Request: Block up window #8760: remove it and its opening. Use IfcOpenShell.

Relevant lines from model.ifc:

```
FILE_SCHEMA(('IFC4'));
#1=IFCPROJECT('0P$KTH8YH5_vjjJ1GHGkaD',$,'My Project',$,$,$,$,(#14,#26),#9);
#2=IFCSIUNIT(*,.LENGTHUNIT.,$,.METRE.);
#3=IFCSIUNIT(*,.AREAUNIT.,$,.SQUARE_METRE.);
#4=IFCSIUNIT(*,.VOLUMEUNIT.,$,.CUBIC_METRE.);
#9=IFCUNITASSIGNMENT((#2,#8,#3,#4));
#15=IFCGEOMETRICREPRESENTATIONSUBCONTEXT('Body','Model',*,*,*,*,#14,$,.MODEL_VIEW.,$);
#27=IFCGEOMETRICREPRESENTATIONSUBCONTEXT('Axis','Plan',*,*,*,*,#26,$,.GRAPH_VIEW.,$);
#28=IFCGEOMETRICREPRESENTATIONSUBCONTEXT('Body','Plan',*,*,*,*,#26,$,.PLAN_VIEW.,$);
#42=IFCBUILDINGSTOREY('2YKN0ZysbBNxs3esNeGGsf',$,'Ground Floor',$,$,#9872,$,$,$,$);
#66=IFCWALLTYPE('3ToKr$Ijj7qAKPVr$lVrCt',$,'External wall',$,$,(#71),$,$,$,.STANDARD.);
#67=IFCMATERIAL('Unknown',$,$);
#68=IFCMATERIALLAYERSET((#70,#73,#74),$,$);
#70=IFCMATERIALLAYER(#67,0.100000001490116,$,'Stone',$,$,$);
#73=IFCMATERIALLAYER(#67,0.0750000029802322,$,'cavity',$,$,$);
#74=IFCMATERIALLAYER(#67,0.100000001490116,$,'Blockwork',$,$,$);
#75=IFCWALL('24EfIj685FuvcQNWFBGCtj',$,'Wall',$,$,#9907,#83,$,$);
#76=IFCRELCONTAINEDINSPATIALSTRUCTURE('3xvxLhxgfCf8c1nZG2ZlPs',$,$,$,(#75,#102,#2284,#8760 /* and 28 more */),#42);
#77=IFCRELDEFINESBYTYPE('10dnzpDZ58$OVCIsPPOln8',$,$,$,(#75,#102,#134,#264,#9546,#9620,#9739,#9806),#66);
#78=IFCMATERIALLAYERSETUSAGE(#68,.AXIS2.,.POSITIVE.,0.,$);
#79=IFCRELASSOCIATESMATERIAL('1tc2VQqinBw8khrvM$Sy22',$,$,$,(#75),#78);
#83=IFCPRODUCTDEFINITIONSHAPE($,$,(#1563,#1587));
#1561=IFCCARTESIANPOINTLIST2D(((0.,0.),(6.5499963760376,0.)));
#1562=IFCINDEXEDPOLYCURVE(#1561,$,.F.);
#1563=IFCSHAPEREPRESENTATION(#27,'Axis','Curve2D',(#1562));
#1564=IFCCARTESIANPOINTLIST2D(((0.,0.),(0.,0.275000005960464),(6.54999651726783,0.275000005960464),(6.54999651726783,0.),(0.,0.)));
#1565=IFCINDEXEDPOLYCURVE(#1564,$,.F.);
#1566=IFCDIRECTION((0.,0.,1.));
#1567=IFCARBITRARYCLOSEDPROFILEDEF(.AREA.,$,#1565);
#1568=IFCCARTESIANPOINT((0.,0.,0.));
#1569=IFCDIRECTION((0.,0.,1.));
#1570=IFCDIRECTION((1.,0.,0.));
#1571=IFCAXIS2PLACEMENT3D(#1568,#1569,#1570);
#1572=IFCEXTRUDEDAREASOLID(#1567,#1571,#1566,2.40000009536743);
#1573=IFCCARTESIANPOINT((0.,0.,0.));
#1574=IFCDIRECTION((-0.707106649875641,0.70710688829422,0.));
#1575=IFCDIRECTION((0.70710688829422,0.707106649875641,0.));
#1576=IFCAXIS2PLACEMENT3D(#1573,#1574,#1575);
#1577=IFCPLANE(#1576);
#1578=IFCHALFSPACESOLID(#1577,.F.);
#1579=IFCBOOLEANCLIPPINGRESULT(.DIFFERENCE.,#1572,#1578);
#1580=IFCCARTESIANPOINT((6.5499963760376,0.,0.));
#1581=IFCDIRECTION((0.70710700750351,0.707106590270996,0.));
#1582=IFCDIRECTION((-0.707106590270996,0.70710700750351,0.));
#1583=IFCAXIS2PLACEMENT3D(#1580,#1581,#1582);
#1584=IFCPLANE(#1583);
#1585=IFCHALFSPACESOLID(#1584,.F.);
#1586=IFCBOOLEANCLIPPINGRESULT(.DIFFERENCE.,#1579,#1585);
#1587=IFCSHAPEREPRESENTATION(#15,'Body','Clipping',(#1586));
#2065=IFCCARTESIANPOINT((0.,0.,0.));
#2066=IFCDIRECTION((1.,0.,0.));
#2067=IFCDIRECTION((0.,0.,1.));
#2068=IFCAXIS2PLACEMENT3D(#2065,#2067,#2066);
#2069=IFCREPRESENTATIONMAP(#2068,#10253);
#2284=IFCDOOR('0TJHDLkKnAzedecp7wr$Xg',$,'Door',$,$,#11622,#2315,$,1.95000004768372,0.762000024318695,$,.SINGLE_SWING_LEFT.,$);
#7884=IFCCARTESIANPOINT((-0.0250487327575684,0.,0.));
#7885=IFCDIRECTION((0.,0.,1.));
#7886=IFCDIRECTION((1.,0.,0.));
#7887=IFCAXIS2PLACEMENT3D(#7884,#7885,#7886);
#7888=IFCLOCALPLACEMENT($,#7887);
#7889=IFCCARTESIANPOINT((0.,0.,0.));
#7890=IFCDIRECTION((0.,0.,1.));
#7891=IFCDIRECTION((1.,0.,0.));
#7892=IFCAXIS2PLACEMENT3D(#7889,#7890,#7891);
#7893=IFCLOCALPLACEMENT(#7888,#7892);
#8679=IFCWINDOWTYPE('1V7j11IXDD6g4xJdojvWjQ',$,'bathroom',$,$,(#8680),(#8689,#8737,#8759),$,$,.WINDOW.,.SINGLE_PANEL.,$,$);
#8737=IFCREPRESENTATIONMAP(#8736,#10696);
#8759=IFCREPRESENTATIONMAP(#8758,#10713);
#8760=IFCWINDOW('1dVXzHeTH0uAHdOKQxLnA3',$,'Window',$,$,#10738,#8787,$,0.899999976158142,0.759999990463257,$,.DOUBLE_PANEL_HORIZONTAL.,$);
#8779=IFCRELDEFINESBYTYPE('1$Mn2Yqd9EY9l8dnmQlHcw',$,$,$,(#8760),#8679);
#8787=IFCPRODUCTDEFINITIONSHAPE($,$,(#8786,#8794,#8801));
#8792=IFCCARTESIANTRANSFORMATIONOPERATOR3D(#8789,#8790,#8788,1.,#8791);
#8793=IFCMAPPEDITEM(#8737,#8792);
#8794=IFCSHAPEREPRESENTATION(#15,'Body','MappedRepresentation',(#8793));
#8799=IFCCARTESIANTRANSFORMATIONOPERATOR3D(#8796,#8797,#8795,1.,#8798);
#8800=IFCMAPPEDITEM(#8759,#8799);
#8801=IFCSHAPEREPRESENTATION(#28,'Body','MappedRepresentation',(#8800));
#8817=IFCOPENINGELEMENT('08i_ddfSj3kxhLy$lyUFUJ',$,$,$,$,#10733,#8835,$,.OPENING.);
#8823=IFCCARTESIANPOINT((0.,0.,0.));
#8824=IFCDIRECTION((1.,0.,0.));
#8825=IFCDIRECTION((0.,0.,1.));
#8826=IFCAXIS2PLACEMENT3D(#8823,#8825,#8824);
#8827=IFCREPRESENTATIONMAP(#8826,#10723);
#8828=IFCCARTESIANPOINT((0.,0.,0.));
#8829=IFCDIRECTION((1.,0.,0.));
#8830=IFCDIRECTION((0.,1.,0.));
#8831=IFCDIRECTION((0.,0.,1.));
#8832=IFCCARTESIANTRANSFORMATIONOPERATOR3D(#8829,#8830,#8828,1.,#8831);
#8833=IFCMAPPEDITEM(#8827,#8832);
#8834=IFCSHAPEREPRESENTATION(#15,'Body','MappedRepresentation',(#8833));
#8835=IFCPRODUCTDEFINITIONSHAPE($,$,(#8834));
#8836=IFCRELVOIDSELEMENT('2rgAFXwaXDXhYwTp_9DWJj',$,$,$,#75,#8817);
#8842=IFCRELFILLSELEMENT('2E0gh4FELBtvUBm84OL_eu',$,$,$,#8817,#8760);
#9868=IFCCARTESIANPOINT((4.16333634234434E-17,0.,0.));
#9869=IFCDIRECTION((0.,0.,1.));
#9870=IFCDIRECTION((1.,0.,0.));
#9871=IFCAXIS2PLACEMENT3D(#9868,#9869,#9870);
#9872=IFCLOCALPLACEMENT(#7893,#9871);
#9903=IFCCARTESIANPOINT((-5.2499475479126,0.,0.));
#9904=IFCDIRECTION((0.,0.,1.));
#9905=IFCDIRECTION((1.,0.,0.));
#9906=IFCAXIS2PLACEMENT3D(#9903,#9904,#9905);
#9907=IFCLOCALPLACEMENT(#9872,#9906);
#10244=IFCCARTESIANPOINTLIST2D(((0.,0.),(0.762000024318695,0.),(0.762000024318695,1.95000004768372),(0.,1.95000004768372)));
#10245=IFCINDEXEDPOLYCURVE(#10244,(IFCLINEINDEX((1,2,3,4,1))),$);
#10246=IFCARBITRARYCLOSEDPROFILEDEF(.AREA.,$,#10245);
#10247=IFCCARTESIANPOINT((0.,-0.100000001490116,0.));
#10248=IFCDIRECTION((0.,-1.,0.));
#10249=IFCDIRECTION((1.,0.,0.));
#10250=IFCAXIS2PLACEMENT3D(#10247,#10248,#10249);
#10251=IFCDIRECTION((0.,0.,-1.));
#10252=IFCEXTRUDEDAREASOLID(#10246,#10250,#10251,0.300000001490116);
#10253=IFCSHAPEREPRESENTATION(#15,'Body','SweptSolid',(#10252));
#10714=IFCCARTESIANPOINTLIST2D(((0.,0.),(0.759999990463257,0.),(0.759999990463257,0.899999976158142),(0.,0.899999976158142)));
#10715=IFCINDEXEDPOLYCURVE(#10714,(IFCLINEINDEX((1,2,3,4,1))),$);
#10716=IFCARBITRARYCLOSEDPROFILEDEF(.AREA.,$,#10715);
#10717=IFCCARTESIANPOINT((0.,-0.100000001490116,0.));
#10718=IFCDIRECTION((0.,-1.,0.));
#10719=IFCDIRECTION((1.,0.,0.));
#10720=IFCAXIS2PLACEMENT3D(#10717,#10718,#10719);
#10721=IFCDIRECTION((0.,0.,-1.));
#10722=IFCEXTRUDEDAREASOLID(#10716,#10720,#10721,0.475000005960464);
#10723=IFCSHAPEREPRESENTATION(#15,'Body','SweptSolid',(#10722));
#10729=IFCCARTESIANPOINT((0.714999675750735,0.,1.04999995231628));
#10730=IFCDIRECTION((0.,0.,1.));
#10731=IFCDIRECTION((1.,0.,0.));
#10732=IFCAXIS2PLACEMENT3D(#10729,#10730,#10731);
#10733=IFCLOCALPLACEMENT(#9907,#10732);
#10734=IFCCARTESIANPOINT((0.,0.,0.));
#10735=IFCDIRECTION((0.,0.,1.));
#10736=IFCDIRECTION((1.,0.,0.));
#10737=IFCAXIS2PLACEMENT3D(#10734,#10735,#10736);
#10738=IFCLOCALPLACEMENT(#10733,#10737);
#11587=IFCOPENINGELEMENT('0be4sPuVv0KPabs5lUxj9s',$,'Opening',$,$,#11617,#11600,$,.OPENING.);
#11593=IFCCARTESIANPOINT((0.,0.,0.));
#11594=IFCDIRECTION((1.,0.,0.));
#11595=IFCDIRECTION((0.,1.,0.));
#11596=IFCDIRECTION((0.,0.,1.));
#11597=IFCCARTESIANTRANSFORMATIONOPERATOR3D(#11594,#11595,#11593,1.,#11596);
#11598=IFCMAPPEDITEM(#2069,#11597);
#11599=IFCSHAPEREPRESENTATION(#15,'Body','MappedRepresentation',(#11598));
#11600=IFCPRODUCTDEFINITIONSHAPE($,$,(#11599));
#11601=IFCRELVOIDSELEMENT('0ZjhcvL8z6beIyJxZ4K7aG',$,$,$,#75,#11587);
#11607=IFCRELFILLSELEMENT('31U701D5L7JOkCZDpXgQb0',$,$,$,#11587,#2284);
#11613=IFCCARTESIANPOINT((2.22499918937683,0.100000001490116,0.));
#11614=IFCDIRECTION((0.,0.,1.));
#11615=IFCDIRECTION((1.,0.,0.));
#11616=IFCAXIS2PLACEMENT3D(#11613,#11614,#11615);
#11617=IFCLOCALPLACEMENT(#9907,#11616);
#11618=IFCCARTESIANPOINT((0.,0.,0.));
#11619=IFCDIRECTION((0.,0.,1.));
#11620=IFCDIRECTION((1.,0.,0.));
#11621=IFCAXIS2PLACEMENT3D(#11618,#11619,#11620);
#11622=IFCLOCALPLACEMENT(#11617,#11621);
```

```python
import ifcopenshell
import ifcopenshell.api.feature
import ifcopenshell.api.root
import ifcopenshell.geom
import ifcopenshell.util.shape

model = ifcopenshell.open("model.ifc")
settings = ifcopenshell.geom.settings()


def volume(element):
    """Net volume in cubic metres, openings subtracted."""
    shape = ifcopenshell.geom.create_shape(settings, element)
    return ifcopenshell.util.shape.get_volume(shape.geometry)


window = model.by_guid("1dVXzHeTH0uAHdOKQxLnA3")
opening = window.FillsVoids[0].RelatingOpeningElement
wall = opening.VoidsElements[0].RelatingBuildingElement
before = volume(wall)

ifcopenshell.api.root.remove_product(model, product=window)
ifcopenshell.api.feature.remove_feature(model, feature=opening)

after = volume(wall)

print(f"wall volume {before:.3f} -> {after:.3f} m3")

model.write("model-out.ifc")
```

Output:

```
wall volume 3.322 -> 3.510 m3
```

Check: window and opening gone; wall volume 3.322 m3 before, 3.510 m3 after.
